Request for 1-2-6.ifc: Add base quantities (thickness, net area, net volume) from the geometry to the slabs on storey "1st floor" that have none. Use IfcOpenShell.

First a look at what the model holds.

```python
import ifcopenshell
import ifcopenshell.util.element
import ifcopenshell.util.unit

model = ifcopenshell.open("1-2-6.ifc")
print(model.schema)
for unit_type in ("LENGTHUNIT", "AREAUNIT", "VOLUMEUNIT"):
    print(unit_type, ifcopenshell.util.unit.calculate_unit_scale(model, unit_type))
storey = next(s for s in model.by_type("IfcBuildingStorey") if s.Name == "1st floor")
slabs = [e for e in ifcopenshell.util.element.get_decomposition(storey) if e.is_a("IfcSlab")]
for e in sorted(slabs, key=lambda e: e.id()):
    print(e.id(), e.is_a(), e.Name, list(ifcopenshell.util.element.get_psets(e, qtos_only=True)), sep=" | ")
```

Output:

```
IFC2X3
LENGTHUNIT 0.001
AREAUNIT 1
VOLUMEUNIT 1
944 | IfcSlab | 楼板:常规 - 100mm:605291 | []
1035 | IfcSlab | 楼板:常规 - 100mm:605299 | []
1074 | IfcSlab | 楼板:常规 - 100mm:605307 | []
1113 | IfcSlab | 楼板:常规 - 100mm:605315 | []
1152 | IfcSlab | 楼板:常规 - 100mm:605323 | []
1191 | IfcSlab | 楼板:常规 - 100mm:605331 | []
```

```python
import ifcopenshell
import ifcopenshell.api.pset
import ifcopenshell.geom
import ifcopenshell.util.element
import ifcopenshell.util.shape
import ifcopenshell.util.unit

model = ifcopenshell.open("1-2-6.ifc")
unit_scale = ifcopenshell.util.unit.calculate_unit_scale(model)
area_scale = ifcopenshell.util.unit.calculate_unit_scale(model, "AREAUNIT")
volume_scale = ifcopenshell.util.unit.calculate_unit_scale(model, "VOLUMEUNIT")
settings = ifcopenshell.geom.settings()

storey = next(s for s in model.by_type("IfcBuildingStorey") if s.Name == "1st floor")
slabs = [e for e in ifcopenshell.util.element.get_decomposition(storey) if e.is_a("IfcSlab")]

for e in sorted(slabs, key=lambda e: e.id()):
    if ifcopenshell.util.element.get_psets(e, qtos_only=True, should_inherit=False):
        continue
    # Geometry comes back in metres, in the element's own axes.
    shape = ifcopenshell.geom.create_shape(settings, e)
    values = {
        "Width": ifcopenshell.util.shape.get_z(shape.geometry) / unit_scale,
        "NetArea": ifcopenshell.util.shape.get_footprint_area(shape.geometry) / area_scale,
        "NetVolume": ifcopenshell.util.shape.get_volume(shape.geometry) / volume_scale,
    }
    qto = ifcopenshell.api.pset.add_qto(model, product=e, name="BaseQuantities")
    ifcopenshell.api.pset.edit_qto(model, qto=qto, properties=values)
    print(e.id(), {k: round(v, 3) for k, v in values.items()})

model.write("1-2-6_v2.ifc")
```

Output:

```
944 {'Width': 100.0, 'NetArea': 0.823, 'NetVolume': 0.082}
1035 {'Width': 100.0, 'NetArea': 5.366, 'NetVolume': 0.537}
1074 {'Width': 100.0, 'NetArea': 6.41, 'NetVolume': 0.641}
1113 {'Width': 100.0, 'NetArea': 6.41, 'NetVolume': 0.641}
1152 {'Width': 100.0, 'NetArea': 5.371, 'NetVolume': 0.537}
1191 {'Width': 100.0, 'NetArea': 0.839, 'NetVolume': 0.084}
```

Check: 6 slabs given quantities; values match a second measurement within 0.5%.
